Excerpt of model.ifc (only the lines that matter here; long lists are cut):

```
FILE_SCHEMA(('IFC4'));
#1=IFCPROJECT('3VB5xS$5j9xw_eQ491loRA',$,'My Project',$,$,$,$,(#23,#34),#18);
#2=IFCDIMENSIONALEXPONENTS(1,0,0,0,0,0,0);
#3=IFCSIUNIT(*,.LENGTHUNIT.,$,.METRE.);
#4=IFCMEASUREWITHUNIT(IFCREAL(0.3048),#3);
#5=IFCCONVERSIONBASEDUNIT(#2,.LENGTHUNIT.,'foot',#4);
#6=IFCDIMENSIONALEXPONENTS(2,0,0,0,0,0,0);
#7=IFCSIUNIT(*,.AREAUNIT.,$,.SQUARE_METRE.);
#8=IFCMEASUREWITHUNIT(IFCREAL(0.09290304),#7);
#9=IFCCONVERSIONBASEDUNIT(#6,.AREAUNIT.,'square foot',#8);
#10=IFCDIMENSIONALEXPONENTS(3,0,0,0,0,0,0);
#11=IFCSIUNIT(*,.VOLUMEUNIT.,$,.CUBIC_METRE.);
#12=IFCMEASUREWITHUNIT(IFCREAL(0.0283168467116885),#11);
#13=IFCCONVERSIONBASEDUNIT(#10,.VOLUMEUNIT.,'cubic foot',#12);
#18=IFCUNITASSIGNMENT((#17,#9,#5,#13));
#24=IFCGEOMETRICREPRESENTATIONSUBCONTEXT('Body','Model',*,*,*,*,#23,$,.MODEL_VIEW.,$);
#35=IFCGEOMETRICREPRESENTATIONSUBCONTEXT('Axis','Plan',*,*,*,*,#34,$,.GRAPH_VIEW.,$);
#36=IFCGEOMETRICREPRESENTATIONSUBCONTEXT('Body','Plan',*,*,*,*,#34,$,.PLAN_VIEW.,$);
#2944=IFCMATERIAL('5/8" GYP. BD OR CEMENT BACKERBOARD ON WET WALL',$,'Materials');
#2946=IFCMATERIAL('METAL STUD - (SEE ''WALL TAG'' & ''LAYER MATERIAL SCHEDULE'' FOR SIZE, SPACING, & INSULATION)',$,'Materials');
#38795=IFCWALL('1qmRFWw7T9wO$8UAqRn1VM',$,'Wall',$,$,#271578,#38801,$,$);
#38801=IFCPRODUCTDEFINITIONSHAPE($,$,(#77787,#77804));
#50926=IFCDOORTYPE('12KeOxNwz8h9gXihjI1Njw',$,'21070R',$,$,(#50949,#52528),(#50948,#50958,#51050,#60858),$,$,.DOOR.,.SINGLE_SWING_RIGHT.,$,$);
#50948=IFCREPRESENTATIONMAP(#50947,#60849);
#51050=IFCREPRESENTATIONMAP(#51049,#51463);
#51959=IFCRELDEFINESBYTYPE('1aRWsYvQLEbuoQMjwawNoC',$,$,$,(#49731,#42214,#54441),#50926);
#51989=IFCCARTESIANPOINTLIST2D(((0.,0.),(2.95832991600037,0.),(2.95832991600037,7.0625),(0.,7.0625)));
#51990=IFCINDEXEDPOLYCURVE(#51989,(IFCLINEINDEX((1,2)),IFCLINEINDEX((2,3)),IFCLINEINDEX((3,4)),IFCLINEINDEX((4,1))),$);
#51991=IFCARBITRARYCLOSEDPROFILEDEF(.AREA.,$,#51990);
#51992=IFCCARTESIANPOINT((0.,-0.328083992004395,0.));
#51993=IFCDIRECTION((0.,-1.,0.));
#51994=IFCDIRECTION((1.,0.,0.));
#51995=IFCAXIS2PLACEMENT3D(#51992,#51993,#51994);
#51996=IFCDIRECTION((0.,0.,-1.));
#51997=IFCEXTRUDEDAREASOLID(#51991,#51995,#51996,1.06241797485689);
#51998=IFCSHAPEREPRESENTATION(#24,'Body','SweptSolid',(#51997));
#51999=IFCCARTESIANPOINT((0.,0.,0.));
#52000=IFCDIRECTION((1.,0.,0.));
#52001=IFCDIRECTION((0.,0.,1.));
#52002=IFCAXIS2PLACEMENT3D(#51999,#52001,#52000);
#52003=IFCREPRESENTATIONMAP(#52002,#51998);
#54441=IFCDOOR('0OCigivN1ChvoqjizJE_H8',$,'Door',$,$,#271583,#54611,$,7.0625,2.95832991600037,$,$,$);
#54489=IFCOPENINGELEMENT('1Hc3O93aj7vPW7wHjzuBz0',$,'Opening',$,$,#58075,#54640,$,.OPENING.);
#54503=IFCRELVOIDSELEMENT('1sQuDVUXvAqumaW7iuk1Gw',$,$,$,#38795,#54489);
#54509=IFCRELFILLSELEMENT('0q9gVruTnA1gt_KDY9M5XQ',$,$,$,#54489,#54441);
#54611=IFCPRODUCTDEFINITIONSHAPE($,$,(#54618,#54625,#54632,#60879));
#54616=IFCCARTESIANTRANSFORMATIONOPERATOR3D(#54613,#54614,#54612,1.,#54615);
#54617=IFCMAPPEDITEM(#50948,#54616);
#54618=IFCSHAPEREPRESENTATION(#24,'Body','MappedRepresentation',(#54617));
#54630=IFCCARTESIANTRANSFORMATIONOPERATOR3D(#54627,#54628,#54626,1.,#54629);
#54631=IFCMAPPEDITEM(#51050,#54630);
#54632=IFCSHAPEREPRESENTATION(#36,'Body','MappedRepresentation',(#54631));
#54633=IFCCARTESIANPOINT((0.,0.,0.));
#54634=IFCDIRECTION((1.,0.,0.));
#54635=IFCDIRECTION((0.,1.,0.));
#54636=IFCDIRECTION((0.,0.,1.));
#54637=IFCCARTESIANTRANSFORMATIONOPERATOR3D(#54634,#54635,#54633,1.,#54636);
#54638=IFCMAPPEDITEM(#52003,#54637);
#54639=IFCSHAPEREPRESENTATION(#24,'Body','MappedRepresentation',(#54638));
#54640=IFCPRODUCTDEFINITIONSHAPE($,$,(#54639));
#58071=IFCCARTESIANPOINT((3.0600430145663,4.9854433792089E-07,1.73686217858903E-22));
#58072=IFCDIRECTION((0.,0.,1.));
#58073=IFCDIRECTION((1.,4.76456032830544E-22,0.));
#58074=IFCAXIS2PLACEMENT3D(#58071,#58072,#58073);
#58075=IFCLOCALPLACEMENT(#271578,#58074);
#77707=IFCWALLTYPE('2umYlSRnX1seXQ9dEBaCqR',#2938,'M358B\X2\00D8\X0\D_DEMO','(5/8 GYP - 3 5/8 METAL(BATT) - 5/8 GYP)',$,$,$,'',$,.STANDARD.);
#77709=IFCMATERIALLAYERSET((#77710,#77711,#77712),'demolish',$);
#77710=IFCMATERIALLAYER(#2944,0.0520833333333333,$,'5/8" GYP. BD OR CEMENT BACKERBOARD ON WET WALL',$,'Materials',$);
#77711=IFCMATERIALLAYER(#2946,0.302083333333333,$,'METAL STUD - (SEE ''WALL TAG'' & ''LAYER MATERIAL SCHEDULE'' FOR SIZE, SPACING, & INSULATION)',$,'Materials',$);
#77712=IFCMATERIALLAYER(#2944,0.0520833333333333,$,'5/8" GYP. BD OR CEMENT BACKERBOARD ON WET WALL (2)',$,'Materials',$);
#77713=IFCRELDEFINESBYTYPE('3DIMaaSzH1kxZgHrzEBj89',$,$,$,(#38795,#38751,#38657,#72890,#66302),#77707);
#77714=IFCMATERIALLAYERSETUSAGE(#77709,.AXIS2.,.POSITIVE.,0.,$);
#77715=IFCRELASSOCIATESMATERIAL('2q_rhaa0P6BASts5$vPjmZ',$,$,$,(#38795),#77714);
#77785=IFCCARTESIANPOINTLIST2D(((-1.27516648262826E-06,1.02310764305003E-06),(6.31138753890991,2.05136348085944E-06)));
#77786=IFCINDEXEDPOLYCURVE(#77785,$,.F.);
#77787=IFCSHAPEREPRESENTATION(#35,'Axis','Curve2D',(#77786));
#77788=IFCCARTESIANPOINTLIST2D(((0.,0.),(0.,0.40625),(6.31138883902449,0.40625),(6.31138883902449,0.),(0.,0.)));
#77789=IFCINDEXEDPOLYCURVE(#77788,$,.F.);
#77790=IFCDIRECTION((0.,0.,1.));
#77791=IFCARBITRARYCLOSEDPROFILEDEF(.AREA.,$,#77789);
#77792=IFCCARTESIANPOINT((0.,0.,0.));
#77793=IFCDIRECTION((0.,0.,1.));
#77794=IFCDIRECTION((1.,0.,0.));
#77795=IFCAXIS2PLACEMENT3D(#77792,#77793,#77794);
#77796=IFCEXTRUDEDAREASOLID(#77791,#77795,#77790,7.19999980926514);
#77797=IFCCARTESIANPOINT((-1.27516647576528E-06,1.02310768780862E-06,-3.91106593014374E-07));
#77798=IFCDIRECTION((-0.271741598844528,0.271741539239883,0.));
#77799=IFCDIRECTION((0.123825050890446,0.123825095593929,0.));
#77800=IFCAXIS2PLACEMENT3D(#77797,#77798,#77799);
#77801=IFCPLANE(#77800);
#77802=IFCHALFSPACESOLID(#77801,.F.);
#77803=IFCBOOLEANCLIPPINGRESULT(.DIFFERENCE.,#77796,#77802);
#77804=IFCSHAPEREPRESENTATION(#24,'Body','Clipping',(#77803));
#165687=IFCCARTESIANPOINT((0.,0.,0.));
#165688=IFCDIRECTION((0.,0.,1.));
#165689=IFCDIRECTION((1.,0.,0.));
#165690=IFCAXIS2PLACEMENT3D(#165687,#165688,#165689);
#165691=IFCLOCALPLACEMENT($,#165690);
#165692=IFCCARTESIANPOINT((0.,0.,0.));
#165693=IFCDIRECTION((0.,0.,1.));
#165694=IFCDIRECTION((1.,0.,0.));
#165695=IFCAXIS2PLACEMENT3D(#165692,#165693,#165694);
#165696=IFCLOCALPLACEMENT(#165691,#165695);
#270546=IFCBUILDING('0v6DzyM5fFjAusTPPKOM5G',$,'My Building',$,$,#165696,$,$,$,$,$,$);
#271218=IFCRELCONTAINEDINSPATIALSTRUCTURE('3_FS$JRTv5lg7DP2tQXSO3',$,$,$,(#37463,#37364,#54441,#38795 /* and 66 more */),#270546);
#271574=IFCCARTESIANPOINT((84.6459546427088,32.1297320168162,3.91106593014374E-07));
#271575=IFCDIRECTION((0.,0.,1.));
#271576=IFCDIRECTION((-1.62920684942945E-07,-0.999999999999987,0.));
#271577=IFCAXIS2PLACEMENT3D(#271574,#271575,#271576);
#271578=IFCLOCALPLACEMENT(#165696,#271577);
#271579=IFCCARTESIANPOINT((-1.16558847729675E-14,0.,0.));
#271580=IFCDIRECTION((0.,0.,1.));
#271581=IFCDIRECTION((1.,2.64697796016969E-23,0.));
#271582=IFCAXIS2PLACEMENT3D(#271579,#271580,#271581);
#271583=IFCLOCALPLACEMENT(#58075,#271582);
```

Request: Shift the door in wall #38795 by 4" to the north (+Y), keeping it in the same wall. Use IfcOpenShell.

```python
import ifcopenshell
import ifcopenshell.api.geometry
import ifcopenshell.util.placement
import ifcopenshell.util.unit

model = ifcopenshell.open("model.ifc")
unit_scale = ifcopenshell.util.unit.calculate_unit_scale(model)

door = model.by_guid("0OCigivN1ChvoqjizJE_H8")
opening = door.FillsVoids[0].RelatingOpeningElement
wall = opening.VoidsElements[0].RelatingBuildingElement

wall_matrix = ifcopenshell.util.placement.get_local_placement(wall.ObjectPlacement)
shift = wall_matrix[:3, 0] * -4 * 0.0254 / unit_scale
before = ifcopenshell.util.placement.get_local_placement(door.ObjectPlacement)[:3, 3].copy()

# The door is placed relative to its opening, so it follows when the opening moves.
matrix = ifcopenshell.util.placement.get_local_placement(opening.ObjectPlacement)
matrix[:3, 3] += shift
ifcopenshell.api.geometry.edit_object_placement(
    model, product=opening, matrix=matrix, is_si=False, should_transform_children=True
)

after = ifcopenshell.util.placement.get_local_placement(door.ObjectPlacement)[:3, 3]
print("door moved by", (after - before).round(3) + 0.0)

model.write("model-out.ifc")
```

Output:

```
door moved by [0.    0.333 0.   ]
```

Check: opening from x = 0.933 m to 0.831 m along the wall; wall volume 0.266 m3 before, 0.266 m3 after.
